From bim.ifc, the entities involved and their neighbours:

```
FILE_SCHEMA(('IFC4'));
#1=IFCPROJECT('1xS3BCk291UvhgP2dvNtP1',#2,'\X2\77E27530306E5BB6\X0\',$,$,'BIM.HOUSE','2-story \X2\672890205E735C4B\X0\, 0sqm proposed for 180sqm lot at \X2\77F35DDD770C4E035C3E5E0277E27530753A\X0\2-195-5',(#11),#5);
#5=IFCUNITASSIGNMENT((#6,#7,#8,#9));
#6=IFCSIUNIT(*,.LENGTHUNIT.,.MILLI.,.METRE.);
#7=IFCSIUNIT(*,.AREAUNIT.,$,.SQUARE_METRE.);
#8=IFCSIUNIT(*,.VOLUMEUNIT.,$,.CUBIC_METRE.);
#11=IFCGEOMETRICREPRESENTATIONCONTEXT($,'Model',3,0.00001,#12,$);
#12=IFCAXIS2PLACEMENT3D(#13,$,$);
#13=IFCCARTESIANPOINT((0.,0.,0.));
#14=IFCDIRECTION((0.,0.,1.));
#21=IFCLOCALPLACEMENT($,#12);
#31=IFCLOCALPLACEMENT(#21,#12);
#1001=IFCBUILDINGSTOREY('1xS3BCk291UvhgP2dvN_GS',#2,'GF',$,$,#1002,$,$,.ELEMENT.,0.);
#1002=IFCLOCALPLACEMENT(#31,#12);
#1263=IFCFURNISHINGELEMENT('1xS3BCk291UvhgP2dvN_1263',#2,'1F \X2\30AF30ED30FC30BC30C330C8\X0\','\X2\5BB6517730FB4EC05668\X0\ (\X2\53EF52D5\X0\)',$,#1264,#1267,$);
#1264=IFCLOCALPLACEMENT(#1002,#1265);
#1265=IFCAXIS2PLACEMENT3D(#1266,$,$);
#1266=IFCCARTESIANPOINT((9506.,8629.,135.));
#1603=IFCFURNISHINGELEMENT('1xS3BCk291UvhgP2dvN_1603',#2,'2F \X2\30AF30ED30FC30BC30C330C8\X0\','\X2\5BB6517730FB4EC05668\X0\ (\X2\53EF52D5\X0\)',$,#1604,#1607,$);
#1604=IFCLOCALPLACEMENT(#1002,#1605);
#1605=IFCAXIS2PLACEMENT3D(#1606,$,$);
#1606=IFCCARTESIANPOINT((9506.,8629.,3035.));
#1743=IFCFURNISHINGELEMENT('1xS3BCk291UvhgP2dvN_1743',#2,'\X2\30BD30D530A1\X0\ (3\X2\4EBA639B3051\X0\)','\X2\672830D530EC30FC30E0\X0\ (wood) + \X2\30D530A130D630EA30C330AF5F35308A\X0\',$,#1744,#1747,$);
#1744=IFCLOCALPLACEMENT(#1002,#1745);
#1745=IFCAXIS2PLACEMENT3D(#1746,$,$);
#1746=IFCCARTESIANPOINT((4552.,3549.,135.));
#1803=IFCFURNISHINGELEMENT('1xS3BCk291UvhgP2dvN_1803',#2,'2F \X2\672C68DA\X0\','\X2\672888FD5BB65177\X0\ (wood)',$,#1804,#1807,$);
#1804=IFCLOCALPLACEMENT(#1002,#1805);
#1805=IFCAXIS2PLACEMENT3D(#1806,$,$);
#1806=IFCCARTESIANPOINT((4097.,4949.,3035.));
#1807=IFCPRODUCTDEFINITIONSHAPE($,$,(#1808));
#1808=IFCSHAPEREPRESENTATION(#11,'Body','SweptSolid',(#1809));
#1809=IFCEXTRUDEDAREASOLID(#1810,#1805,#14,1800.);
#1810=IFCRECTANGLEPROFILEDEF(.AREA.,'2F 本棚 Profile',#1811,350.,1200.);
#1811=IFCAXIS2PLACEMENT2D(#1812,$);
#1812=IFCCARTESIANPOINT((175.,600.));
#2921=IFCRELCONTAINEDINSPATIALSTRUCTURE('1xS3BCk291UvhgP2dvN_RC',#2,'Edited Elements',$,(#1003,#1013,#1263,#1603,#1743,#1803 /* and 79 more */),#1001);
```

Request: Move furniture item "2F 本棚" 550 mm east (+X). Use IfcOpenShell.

```python
import ifcopenshell
import ifcopenshell.api.geometry
import ifcopenshell.util.placement
import ifcopenshell.util.unit

model = ifcopenshell.open("bim.ifc")
unit_scale = ifcopenshell.util.unit.calculate_unit_scale(model)

item = model.by_id(1803)
matrix = ifcopenshell.util.placement.get_local_placement(item.ObjectPlacement)
matrix[0, 3] += 0.55 / unit_scale
ifcopenshell.api.geometry.edit_object_placement(model, product=item, matrix=matrix, is_si=False)

print(ifcopenshell.util.placement.get_local_placement(item.ObjectPlacement).round(3) + 0.0)

model.write("bim-out.ifc")
```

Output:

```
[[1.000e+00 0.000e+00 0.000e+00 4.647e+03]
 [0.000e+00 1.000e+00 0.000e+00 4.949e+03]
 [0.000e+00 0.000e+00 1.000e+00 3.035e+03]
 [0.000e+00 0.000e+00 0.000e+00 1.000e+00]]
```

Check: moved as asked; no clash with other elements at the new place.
